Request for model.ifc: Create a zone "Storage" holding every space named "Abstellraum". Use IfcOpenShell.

First a look at what the model holds.

```python
import ifcopenshell

model = ifcopenshell.open("model.ifc")
print(model.schema)
seen = {}
for space in model.by_type("IfcSpace"):
    seen[space.LongName] = seen.get(space.LongName, 0) + 1
for name, count in sorted(seen.items(), key=str):
    print(count, "x", name)
print("zones:", [z.Name for z in model.by_type("IfcZone")][:20])
```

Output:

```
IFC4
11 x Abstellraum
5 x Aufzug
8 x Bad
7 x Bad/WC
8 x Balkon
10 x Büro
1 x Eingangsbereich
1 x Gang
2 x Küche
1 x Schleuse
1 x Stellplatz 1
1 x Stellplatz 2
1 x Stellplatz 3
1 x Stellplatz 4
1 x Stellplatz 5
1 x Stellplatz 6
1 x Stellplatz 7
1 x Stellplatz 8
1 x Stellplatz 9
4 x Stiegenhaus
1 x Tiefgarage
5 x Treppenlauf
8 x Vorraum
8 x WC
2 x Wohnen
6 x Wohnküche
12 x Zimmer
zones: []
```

```python
import ifcopenshell
import ifcopenshell.api.group
import ifcopenshell.api.root

model = ifcopenshell.open("model.ifc")

names = {"Abstellraum"}
spaces = [s for s in model.by_type("IfcSpace") if s.LongName in names]

zone = ifcopenshell.api.root.create_entity(model, ifc_class="IfcZone", name="Storage")
ifcopenshell.api.group.assign_group(model, products=spaces, group=zone)
print(len(spaces), "spaces in", zone.Name)

model.write("model_edited.ifc")
```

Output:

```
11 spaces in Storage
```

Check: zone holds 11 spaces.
